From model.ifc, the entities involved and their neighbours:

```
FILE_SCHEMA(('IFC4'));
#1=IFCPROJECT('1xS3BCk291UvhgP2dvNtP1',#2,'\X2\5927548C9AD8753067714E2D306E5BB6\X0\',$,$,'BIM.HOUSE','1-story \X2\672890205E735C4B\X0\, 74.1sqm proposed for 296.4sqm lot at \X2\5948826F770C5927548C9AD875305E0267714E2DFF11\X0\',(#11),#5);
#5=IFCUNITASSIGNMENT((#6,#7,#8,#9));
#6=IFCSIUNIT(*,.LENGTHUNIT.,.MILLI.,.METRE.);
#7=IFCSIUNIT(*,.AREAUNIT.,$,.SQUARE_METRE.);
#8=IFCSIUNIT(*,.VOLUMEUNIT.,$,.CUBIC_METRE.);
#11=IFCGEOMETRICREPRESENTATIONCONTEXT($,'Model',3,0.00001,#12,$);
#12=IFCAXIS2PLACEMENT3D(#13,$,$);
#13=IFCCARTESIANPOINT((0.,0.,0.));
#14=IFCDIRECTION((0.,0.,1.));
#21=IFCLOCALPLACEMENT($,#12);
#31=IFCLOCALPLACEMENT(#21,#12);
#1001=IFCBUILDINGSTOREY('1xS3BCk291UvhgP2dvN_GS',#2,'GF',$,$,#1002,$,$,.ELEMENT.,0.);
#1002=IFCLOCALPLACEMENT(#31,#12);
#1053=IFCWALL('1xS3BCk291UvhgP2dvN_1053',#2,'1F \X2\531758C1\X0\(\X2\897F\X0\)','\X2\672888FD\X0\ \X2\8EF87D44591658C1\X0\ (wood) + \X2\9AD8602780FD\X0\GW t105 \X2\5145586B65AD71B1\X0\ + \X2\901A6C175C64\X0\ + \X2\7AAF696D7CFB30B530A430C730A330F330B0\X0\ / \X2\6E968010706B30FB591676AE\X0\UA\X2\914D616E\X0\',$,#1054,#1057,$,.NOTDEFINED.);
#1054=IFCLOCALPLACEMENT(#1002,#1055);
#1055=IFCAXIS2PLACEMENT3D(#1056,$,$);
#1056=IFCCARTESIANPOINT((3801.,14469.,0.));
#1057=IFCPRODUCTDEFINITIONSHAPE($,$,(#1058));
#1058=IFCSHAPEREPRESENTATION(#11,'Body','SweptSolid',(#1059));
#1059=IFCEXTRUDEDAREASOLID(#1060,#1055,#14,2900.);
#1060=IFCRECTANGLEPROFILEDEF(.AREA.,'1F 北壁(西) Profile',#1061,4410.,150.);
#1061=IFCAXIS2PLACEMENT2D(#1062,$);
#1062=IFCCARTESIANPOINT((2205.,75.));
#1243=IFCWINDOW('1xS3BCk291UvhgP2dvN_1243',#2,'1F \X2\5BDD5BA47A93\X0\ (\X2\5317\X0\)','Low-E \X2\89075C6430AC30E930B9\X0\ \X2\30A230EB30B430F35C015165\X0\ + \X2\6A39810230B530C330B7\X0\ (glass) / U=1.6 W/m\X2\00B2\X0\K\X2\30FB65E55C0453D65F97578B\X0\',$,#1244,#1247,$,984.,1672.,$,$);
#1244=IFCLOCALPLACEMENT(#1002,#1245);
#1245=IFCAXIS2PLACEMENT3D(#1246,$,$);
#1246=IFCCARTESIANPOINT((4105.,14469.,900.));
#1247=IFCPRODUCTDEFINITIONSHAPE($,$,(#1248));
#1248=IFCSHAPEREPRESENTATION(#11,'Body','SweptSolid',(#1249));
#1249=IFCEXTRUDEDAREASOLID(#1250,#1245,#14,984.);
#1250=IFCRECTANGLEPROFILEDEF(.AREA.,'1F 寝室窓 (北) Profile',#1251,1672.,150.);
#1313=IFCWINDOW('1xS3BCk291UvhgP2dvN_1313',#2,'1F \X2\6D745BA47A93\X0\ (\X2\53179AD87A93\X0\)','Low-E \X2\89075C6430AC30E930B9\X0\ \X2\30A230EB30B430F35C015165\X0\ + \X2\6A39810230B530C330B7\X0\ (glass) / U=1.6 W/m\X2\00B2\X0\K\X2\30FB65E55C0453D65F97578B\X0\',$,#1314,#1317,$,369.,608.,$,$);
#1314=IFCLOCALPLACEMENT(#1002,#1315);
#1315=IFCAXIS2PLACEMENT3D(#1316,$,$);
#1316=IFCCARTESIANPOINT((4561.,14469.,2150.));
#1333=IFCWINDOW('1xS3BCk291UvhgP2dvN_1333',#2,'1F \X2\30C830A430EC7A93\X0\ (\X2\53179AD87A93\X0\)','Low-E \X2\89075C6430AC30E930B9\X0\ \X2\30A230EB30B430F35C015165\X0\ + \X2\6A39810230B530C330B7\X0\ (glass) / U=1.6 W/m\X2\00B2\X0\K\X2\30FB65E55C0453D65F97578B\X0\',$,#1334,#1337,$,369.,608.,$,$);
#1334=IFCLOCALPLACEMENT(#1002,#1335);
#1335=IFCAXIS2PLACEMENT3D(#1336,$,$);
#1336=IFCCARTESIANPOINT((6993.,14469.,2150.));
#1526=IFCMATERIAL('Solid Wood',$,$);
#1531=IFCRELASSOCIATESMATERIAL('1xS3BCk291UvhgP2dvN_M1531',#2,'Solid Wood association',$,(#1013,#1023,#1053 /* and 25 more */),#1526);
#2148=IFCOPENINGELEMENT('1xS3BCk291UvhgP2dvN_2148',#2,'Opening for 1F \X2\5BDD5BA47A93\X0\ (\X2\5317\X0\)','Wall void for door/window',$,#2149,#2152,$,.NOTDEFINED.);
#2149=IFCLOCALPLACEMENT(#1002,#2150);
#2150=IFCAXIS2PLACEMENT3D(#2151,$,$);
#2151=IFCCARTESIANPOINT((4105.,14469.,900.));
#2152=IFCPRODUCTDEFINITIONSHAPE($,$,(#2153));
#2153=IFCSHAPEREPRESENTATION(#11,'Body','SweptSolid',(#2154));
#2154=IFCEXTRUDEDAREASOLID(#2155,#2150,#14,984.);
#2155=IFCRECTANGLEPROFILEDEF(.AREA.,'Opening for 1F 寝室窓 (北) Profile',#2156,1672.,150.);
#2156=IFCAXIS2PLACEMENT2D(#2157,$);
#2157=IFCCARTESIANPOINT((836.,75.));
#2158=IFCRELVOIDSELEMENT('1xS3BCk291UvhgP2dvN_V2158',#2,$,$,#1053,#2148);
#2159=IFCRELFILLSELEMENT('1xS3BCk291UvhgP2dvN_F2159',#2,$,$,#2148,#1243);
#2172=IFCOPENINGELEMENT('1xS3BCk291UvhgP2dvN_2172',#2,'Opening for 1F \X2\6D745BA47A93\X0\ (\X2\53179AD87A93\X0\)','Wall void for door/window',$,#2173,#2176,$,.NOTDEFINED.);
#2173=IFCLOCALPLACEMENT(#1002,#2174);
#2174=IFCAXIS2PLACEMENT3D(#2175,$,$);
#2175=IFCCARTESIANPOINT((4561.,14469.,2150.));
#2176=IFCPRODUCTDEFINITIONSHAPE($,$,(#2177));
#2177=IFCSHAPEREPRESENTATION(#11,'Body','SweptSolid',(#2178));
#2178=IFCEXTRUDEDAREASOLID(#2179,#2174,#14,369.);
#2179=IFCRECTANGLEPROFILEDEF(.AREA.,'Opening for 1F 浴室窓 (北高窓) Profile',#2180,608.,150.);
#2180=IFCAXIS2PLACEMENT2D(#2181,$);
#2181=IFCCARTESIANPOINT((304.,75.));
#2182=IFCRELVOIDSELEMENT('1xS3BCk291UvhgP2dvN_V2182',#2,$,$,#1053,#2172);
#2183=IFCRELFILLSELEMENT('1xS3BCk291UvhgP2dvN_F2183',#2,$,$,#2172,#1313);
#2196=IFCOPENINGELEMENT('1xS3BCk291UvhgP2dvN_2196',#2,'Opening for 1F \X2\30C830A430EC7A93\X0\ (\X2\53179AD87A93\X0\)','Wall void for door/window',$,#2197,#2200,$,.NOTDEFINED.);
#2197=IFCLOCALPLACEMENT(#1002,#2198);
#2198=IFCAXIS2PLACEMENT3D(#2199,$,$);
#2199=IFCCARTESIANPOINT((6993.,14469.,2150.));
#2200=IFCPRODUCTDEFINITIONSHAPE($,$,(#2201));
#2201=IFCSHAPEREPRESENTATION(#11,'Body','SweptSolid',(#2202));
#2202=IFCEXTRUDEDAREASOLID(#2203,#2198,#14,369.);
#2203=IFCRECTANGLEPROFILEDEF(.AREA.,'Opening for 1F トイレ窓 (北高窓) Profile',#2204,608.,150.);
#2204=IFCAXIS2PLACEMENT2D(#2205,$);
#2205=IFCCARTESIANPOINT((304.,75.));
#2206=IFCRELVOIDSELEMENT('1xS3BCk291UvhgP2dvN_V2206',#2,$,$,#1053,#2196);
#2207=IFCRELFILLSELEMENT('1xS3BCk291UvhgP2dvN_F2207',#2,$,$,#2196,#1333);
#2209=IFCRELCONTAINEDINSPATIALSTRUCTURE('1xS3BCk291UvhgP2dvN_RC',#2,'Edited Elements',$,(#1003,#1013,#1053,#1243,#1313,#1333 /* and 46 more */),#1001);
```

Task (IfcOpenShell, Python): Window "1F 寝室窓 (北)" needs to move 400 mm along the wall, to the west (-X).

```python
import ifcopenshell
import ifcopenshell.api.geometry
import ifcopenshell.util.placement

model = ifcopenshell.open("model.ifc")

window = model.by_guid("1xS3BCk291UvhgP2dvN_1243")
opening = window.FillsVoids[0].RelatingOpeningElement
wall = opening.VoidsElements[0].RelatingBuildingElement

wall_matrix = ifcopenshell.util.placement.get_local_placement(wall.ObjectPlacement)
shift = wall_matrix[:3, 0] * -400.0
before = ifcopenshell.util.placement.get_local_placement(window.ObjectPlacement)[:3, 3].copy()

# The window is not placed relative to its opening, so move both.
for product in (opening, window):
    matrix = ifcopenshell.util.placement.get_local_placement(product.ObjectPlacement)
    matrix[:3, 3] += shift
    ifcopenshell.api.geometry.edit_object_placement(model, product=product, matrix=matrix, is_si=False)

after = ifcopenshell.util.placement.get_local_placement(window.ObjectPlacement)[:3, 3]
print("window moved by", (after - before).round(3) + 0.0)

model.write("model_rev.ifc")
```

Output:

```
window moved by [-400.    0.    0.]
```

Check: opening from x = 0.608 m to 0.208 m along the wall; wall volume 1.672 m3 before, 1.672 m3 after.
